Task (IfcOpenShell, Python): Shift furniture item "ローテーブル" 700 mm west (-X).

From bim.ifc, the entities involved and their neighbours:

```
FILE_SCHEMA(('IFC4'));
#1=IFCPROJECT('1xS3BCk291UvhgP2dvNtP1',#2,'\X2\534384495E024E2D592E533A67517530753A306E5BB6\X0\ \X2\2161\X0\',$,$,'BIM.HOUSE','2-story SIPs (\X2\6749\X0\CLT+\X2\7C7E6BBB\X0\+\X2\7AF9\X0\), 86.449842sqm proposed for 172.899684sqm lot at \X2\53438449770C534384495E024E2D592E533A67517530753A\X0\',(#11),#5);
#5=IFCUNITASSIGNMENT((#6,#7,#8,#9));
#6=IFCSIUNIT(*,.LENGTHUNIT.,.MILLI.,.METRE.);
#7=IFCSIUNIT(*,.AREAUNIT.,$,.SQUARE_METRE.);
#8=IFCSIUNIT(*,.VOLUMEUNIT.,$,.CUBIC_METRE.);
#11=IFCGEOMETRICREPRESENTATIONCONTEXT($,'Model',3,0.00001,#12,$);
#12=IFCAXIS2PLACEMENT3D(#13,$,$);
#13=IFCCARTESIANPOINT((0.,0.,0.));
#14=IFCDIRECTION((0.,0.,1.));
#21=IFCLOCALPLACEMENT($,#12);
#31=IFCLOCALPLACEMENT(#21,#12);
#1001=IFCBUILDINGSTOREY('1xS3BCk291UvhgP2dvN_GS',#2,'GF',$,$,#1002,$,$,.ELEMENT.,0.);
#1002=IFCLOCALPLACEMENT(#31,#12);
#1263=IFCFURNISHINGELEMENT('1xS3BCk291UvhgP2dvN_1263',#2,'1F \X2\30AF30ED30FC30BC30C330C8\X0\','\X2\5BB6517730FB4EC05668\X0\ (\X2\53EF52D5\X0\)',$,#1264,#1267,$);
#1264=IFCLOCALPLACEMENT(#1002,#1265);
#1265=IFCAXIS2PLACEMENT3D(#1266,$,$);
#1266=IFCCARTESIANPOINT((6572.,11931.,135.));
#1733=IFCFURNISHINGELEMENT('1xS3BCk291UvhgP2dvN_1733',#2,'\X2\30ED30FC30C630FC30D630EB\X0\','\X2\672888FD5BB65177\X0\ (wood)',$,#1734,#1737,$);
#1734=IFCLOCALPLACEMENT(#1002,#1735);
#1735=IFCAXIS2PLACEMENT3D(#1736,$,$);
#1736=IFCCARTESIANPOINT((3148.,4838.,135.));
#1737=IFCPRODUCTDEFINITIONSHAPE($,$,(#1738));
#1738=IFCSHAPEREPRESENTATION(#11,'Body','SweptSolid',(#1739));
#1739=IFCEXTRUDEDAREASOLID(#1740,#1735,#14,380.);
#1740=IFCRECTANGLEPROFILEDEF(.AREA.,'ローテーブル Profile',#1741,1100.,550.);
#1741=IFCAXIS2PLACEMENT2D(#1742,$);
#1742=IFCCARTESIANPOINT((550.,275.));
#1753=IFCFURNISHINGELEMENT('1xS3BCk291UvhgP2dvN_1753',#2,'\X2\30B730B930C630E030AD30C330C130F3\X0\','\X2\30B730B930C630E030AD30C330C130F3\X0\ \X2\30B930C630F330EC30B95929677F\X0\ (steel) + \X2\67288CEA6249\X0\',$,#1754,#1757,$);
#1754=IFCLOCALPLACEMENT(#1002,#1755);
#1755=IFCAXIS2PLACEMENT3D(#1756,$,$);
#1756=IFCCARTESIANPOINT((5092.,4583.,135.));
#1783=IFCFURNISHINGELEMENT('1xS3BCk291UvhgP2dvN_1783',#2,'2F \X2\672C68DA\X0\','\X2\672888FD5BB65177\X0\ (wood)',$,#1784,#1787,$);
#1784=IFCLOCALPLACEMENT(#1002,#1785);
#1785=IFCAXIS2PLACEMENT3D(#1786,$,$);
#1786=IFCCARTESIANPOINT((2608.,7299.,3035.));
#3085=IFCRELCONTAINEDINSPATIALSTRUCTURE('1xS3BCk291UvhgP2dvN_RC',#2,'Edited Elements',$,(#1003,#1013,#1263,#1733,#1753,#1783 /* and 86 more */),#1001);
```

```python
import ifcopenshell
import ifcopenshell.api.geometry
import ifcopenshell.util.placement
import ifcopenshell.util.unit

model = ifcopenshell.open("bim.ifc")
unit_scale = ifcopenshell.util.unit.calculate_unit_scale(model)

item = model.by_guid("1xS3BCk291UvhgP2dvN_1733")
matrix = ifcopenshell.util.placement.get_local_placement(item.ObjectPlacement)
matrix[0, 3] -= 0.7 / unit_scale
ifcopenshell.api.geometry.edit_object_placement(model, product=item, matrix=matrix, is_si=False)

print(ifcopenshell.util.placement.get_local_placement(item.ObjectPlacement).round(3) + 0.0)

model.write("bim_updated.ifc")
```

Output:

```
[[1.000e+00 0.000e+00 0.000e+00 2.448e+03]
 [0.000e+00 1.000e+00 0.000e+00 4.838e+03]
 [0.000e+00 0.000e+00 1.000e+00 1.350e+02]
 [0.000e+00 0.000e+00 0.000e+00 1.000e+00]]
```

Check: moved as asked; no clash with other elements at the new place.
